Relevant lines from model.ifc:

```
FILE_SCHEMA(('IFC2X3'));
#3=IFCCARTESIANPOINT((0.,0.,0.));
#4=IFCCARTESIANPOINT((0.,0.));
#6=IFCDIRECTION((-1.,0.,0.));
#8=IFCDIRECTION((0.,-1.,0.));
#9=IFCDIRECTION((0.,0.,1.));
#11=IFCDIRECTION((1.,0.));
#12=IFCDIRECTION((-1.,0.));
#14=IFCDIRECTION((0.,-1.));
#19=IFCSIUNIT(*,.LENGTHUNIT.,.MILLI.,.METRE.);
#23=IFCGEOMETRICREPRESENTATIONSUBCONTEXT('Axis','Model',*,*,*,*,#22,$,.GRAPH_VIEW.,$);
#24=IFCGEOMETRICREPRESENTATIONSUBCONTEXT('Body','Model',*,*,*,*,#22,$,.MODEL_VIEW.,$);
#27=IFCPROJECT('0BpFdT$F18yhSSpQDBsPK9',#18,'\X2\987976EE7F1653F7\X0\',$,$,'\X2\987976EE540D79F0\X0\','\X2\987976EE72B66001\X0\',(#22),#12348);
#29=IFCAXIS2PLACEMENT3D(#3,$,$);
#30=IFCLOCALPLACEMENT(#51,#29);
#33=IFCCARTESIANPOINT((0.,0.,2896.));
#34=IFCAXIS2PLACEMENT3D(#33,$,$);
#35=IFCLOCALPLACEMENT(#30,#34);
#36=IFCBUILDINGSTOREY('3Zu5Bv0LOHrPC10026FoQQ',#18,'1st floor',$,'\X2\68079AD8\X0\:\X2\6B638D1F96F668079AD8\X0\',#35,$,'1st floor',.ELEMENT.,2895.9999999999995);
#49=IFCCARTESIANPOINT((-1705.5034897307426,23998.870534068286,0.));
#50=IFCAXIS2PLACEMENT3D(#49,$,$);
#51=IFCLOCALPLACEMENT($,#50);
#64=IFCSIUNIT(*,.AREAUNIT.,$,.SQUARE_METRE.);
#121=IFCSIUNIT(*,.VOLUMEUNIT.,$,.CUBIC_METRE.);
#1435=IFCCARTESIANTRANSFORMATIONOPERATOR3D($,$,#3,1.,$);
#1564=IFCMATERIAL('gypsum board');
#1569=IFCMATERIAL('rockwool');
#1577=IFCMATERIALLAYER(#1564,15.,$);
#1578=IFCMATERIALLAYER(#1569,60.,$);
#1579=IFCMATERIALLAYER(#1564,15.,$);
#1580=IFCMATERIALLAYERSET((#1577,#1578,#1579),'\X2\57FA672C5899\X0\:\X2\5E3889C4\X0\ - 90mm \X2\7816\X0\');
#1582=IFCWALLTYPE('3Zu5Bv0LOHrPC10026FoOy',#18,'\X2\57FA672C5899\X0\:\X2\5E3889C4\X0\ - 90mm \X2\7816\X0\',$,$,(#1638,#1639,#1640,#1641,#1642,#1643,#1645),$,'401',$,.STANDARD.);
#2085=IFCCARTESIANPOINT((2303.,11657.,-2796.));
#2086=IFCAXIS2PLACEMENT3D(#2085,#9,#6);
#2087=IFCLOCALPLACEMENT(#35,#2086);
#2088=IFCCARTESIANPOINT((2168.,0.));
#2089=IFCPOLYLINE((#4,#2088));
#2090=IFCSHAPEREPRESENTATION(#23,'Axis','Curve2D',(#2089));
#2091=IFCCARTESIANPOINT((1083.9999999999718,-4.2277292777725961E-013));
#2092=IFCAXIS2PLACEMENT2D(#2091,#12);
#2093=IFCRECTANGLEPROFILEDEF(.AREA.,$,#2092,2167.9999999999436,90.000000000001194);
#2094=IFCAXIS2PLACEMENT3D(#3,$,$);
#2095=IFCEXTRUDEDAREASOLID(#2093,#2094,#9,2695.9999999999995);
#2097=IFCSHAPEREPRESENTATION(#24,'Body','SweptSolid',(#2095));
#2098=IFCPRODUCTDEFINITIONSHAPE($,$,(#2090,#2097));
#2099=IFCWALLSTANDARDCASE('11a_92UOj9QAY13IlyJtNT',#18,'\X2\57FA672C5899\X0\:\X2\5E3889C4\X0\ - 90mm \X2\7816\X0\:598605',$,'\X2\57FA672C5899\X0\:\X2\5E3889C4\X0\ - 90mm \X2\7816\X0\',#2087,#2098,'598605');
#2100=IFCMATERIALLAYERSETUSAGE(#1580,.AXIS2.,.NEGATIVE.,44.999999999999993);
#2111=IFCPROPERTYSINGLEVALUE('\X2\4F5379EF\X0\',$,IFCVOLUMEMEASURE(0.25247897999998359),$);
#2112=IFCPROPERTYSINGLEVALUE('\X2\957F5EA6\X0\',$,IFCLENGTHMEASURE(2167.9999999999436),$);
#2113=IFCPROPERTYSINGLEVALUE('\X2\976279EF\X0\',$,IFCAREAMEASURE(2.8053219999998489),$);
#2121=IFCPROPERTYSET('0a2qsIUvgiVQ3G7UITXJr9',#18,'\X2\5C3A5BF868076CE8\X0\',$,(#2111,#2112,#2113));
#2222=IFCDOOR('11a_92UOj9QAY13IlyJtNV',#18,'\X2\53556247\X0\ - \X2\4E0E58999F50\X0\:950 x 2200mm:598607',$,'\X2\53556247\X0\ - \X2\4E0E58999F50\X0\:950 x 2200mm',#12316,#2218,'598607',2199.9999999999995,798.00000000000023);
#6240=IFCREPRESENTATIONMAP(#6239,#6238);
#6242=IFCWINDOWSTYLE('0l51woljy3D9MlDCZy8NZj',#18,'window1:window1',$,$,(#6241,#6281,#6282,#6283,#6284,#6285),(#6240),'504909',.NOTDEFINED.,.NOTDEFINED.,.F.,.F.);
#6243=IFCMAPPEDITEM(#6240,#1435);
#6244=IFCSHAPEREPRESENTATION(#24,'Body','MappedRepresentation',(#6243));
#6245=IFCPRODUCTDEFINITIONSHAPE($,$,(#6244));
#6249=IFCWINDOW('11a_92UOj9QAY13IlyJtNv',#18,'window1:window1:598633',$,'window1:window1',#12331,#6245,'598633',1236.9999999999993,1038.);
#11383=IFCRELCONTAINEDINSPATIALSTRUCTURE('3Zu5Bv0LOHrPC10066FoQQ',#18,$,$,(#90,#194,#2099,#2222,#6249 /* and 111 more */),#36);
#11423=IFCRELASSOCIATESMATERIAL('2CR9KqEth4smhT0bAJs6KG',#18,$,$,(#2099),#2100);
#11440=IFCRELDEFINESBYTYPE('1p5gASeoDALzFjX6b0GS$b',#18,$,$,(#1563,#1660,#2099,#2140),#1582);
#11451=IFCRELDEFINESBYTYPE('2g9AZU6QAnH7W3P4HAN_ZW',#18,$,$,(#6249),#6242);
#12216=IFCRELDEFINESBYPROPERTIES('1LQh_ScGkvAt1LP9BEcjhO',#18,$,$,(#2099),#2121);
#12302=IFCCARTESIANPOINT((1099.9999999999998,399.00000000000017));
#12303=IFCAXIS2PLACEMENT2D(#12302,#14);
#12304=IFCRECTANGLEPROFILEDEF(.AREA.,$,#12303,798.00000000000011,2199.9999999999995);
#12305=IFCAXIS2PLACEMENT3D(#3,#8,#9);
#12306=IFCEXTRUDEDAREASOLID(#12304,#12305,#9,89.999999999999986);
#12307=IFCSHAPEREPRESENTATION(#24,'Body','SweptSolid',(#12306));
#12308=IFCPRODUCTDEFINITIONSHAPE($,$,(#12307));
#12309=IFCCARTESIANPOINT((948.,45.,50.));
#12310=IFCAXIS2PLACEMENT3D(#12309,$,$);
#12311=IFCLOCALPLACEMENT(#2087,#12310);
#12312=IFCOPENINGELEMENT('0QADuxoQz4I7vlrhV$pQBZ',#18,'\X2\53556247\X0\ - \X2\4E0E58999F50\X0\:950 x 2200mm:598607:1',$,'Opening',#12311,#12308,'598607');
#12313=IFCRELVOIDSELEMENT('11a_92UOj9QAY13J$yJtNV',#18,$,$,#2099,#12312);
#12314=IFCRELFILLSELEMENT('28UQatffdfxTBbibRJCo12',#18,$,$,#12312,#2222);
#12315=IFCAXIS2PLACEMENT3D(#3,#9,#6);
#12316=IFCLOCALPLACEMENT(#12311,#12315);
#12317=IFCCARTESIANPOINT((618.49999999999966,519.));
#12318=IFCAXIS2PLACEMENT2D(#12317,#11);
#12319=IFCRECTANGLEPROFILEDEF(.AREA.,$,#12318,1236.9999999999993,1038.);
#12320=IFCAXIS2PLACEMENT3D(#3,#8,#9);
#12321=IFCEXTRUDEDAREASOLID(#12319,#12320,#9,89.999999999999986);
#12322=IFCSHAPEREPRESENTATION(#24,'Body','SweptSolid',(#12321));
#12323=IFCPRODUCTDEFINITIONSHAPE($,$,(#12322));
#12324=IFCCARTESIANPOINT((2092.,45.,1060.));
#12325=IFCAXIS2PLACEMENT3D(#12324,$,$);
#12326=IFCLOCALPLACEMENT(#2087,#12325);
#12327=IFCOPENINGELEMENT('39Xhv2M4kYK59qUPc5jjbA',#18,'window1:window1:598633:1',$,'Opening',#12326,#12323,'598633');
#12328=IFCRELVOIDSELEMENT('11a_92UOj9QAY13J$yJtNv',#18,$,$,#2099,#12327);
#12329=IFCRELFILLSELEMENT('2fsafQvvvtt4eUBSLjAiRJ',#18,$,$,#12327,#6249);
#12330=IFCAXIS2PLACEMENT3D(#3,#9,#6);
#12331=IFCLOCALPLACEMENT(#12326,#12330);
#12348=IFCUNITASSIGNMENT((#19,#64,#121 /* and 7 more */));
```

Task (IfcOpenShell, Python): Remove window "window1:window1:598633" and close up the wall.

```python
import ifcopenshell
import ifcopenshell.api.feature
import ifcopenshell.api.pset
import ifcopenshell.api.root
import ifcopenshell.geom
import ifcopenshell.util.element
import ifcopenshell.util.shape
import ifcopenshell.util.unit

model = ifcopenshell.open("model.ifc")
area_scale = ifcopenshell.util.unit.calculate_unit_scale(model, "AREAUNIT")
volume_scale = ifcopenshell.util.unit.calculate_unit_scale(model, "VOLUMEUNIT")
settings = ifcopenshell.geom.settings()


def volume(element):
    """Net volume in cubic metres, openings subtracted."""
    shape = ifcopenshell.geom.create_shape(settings, element)
    return ifcopenshell.util.shape.get_volume(shape.geometry)


window = model.by_guid("11a_92UOj9QAY13IlyJtNv")
opening = window.FillsVoids[0].RelatingOpeningElement
wall = opening.VoidsElements[0].RelatingBuildingElement
before = volume(wall)

ifcopenshell.api.root.remove_product(model, product=window)
ifcopenshell.api.feature.remove_feature(model, feature=opening)

after = volume(wall)
thickness = 0.09  # wall thickness in metres

# Update the wall's stored quantities.
pset = model.by_id(ifcopenshell.util.element.get_pset(wall, "尺寸标注", should_inherit=False)["id"])
ifcopenshell.api.pset.edit_pset(model, pset=pset, properties={
    "体积": model.create_entity("IfcVolumeMeasure", after / volume_scale),
    "面积": model.create_entity("IfcAreaMeasure", after / thickness / area_scale),
})

print(f"wall volume {before:.3f} -> {after:.3f} m3")

model.write("model_rev.ifc")
```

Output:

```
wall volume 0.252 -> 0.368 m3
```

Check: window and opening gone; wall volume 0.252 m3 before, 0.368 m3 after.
